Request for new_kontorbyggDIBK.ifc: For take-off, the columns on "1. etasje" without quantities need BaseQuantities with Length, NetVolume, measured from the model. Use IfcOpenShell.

First a look at what the model holds.

```python
import ifcopenshell
import ifcopenshell.util.element
import ifcopenshell.util.unit

model = ifcopenshell.open("new_kontorbyggDIBK.ifc")
print(model.schema)
for unit_type in ("LENGTHUNIT", "AREAUNIT", "VOLUMEUNIT"):
    print(unit_type, ifcopenshell.util.unit.calculate_unit_scale(model, unit_type))
storey = next(s for s in model.by_type("IfcBuildingStorey") if s.Name == "1. etasje")
columns = [e for e in ifcopenshell.util.element.get_decomposition(storey) if e.is_a("IfcColumn")]
for e in sorted(columns, key=lambda e: e.id()):
    print(e.id(), e.is_a(), e.Name, list(ifcopenshell.util.element.get_psets(e, qtos_only=True)), sep=" | ")
```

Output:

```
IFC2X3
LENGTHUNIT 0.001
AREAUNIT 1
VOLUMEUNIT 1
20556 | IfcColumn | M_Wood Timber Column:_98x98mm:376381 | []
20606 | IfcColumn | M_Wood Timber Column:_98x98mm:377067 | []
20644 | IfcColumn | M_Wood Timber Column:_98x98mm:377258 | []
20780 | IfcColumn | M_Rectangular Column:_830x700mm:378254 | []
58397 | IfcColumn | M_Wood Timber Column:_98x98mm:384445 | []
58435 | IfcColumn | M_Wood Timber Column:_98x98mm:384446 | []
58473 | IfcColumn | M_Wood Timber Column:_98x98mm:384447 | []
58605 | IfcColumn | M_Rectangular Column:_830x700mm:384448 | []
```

```python
import ifcopenshell
import ifcopenshell.api.pset
import ifcopenshell.geom
import ifcopenshell.util.element
import ifcopenshell.util.shape
import ifcopenshell.util.unit

model = ifcopenshell.open("new_kontorbyggDIBK.ifc")
unit_scale = ifcopenshell.util.unit.calculate_unit_scale(model)
volume_scale = ifcopenshell.util.unit.calculate_unit_scale(model, "VOLUMEUNIT")
settings = ifcopenshell.geom.settings()

storey = next(s for s in model.by_type("IfcBuildingStorey") if s.Name == "1. etasje")
columns = [e for e in ifcopenshell.util.element.get_decomposition(storey) if e.is_a("IfcColumn")]

for e in sorted(columns, key=lambda e: e.id()):
    if ifcopenshell.util.element.get_psets(e, qtos_only=True, should_inherit=False):
        continue
    # Geometry comes back in metres, in the element's own axes.
    shape = ifcopenshell.geom.create_shape(settings, e)
    values = {
        "Length": ifcopenshell.util.shape.get_z(shape.geometry) / unit_scale,
        "NetVolume": ifcopenshell.util.shape.get_volume(shape.geometry) / volume_scale,
    }
    qto = ifcopenshell.api.pset.add_qto(model, product=e, name="BaseQuantities")
    ifcopenshell.api.pset.edit_qto(model, qto=qto, properties=values)
    print(e.id(), {k: round(v, 3) for k, v in values.items()})

model.write("new_kontorbyggDIBK_v2.ifc")
```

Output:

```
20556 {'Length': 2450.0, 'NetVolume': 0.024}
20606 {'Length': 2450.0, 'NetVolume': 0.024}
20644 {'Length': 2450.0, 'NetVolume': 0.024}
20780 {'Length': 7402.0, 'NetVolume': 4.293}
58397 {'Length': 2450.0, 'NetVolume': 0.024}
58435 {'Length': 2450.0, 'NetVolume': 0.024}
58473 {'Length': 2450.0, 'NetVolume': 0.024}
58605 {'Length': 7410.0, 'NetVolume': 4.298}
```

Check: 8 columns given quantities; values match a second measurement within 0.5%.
